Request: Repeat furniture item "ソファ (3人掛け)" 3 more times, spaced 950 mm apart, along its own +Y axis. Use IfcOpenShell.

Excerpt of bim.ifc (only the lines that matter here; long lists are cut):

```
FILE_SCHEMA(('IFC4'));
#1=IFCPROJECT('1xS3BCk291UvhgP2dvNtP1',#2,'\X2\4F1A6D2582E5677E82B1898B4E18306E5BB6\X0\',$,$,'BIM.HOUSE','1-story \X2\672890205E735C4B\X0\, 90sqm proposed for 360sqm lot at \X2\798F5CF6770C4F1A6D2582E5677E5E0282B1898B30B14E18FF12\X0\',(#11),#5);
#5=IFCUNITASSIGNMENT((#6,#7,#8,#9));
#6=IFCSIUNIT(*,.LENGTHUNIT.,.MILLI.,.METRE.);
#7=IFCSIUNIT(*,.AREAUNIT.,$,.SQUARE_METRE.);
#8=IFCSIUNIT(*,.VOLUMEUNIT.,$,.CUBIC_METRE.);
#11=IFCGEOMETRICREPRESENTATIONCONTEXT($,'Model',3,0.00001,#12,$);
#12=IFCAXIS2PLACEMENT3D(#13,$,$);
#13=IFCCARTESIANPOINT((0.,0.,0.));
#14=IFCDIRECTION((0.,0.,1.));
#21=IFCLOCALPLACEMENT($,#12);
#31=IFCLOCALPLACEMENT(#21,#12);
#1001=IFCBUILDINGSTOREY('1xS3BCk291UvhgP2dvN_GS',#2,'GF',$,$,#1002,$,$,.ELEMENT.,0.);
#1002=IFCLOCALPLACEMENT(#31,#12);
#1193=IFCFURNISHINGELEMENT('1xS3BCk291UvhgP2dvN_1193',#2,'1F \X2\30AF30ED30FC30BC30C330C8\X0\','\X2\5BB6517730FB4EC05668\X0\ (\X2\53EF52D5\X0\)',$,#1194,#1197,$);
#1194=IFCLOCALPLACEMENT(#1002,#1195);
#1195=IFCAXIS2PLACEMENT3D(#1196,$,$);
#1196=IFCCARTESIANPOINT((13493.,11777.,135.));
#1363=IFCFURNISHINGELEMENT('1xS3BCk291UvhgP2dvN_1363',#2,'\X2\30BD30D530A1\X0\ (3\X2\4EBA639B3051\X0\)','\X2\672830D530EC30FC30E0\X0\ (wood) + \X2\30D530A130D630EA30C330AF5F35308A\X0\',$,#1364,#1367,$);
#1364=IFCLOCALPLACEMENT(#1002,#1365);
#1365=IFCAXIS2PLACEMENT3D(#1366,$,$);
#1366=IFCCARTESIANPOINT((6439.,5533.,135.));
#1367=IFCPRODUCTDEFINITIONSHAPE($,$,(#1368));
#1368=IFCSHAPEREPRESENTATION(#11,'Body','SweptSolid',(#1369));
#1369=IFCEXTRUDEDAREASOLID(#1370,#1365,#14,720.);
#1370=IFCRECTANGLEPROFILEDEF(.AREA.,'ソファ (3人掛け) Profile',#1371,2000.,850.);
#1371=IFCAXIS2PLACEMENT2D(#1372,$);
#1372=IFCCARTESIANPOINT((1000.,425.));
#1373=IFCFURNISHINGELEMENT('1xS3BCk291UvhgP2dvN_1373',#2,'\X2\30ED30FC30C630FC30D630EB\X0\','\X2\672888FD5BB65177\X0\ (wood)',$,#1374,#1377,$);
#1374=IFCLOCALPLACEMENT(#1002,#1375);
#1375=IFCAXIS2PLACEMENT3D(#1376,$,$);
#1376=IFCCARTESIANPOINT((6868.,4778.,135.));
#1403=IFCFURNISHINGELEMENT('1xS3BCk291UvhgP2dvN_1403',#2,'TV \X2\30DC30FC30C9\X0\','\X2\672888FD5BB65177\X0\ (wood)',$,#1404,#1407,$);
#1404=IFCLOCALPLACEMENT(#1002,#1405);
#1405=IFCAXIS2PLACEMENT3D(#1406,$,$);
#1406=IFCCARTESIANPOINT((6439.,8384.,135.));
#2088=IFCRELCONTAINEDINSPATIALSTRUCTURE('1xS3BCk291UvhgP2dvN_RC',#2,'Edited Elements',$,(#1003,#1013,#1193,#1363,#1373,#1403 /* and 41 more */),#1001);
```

```python
import ifcopenshell
import ifcopenshell.api.geometry
import ifcopenshell.api.root
import ifcopenshell.util.element
import ifcopenshell.util.placement

model = ifcopenshell.open("bim.ifc")


def reuse_history(source, copy):
    """copy_class also copies each property set's owner history, people and application; keep the originals."""
    for rel in copy.IsDefinedBy:
        if rel.is_a("IfcRelDefinesByProperties") and (history := rel.RelatingPropertyDefinition.OwnerHistory):
            rel.RelatingPropertyDefinition.OwnerHistory = source.OwnerHistory
            ifcopenshell.util.element.remove_deep2(model, history)


source = model.by_guid("1xS3BCk291UvhgP2dvN_1363")
base = ifcopenshell.util.placement.get_local_placement(source.ObjectPlacement)
step = base[:3, 1] * 950.0

for i in range(1, 4):
    copy = ifcopenshell.api.root.copy_class(model, product=source)
    copy.Representation = ifcopenshell.util.element.copy_deep(
        model, source.Representation, exclude=["IfcGeometricRepresentationContext", "IfcRepresentationMap"]
    )
    reuse_history(source, copy)
    matrix = base.copy()
    matrix[:3, 3] += i * step
    print("added at", matrix[:3, 3].round(3) + 0.0)
    ifcopenshell.api.geometry.edit_object_placement(model, product=copy, matrix=matrix, is_si=False)

model.write("bim_v2.ifc")
```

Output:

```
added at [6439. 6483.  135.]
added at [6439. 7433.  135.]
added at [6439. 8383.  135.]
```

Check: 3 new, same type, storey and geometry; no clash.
